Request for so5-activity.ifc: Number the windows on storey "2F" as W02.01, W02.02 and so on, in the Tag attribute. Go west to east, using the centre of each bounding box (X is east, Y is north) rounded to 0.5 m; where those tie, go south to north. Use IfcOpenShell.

First a look at what the model holds.

```python
import ifcopenshell
import ifcopenshell.util.element
import ifcopenshell.util.placement

model = ifcopenshell.open("so5-activity.ifc")
print(model.schema)
storey = next(s for s in model.by_type("IfcBuildingStorey") if s.Name == "2F")
windows = [e for e in ifcopenshell.util.element.get_decomposition(storey) if e.is_a("IfcWindow")]
for e in sorted(windows, key=lambda e: e.id()):
    origin = ifcopenshell.util.placement.get_local_placement(e.ObjectPlacement)[:3, 3]
    print(e.id(), e.Tag, e.Name, origin.round(2) + 0.0, sep=" | ")
```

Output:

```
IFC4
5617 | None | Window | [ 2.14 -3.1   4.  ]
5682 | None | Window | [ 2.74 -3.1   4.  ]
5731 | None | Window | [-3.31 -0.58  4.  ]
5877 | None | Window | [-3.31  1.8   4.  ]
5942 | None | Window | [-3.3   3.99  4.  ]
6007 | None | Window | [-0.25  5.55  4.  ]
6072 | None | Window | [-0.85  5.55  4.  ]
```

```python
import ifcopenshell
import ifcopenshell.geom
import ifcopenshell.util.element
import ifcopenshell.util.shape

model = ifcopenshell.open("so5-activity.ifc")
settings = ifcopenshell.geom.settings()
settings.set("use-world-coords", True)


def centre(element):
    shape = ifcopenshell.geom.create_shape(settings, element)
    return ifcopenshell.util.shape.get_bbox_centroid(shape.geometry)


storey = next(s for s in model.by_type("IfcBuildingStorey") if s.Name == "2F")
windows = [e for e in ifcopenshell.util.element.get_decomposition(storey) if e.is_a("IfcWindow")]

# Insertion points can sit at a corner or the storey origin, so sort by the geometry (in metres).
centres = {e: centre(e) for e in windows}
windows.sort(key=lambda e: (round(centres[e][0] / 0.5), centres[e][1]))

for i, e in enumerate(windows, start=1):
    number = f"W02.{i:02d}"
    e.Tag = number
    print(e.id(), number)

model.write("so5-activity_updated.ifc")
```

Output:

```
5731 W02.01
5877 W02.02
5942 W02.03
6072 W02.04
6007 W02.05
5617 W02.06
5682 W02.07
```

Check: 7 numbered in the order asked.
